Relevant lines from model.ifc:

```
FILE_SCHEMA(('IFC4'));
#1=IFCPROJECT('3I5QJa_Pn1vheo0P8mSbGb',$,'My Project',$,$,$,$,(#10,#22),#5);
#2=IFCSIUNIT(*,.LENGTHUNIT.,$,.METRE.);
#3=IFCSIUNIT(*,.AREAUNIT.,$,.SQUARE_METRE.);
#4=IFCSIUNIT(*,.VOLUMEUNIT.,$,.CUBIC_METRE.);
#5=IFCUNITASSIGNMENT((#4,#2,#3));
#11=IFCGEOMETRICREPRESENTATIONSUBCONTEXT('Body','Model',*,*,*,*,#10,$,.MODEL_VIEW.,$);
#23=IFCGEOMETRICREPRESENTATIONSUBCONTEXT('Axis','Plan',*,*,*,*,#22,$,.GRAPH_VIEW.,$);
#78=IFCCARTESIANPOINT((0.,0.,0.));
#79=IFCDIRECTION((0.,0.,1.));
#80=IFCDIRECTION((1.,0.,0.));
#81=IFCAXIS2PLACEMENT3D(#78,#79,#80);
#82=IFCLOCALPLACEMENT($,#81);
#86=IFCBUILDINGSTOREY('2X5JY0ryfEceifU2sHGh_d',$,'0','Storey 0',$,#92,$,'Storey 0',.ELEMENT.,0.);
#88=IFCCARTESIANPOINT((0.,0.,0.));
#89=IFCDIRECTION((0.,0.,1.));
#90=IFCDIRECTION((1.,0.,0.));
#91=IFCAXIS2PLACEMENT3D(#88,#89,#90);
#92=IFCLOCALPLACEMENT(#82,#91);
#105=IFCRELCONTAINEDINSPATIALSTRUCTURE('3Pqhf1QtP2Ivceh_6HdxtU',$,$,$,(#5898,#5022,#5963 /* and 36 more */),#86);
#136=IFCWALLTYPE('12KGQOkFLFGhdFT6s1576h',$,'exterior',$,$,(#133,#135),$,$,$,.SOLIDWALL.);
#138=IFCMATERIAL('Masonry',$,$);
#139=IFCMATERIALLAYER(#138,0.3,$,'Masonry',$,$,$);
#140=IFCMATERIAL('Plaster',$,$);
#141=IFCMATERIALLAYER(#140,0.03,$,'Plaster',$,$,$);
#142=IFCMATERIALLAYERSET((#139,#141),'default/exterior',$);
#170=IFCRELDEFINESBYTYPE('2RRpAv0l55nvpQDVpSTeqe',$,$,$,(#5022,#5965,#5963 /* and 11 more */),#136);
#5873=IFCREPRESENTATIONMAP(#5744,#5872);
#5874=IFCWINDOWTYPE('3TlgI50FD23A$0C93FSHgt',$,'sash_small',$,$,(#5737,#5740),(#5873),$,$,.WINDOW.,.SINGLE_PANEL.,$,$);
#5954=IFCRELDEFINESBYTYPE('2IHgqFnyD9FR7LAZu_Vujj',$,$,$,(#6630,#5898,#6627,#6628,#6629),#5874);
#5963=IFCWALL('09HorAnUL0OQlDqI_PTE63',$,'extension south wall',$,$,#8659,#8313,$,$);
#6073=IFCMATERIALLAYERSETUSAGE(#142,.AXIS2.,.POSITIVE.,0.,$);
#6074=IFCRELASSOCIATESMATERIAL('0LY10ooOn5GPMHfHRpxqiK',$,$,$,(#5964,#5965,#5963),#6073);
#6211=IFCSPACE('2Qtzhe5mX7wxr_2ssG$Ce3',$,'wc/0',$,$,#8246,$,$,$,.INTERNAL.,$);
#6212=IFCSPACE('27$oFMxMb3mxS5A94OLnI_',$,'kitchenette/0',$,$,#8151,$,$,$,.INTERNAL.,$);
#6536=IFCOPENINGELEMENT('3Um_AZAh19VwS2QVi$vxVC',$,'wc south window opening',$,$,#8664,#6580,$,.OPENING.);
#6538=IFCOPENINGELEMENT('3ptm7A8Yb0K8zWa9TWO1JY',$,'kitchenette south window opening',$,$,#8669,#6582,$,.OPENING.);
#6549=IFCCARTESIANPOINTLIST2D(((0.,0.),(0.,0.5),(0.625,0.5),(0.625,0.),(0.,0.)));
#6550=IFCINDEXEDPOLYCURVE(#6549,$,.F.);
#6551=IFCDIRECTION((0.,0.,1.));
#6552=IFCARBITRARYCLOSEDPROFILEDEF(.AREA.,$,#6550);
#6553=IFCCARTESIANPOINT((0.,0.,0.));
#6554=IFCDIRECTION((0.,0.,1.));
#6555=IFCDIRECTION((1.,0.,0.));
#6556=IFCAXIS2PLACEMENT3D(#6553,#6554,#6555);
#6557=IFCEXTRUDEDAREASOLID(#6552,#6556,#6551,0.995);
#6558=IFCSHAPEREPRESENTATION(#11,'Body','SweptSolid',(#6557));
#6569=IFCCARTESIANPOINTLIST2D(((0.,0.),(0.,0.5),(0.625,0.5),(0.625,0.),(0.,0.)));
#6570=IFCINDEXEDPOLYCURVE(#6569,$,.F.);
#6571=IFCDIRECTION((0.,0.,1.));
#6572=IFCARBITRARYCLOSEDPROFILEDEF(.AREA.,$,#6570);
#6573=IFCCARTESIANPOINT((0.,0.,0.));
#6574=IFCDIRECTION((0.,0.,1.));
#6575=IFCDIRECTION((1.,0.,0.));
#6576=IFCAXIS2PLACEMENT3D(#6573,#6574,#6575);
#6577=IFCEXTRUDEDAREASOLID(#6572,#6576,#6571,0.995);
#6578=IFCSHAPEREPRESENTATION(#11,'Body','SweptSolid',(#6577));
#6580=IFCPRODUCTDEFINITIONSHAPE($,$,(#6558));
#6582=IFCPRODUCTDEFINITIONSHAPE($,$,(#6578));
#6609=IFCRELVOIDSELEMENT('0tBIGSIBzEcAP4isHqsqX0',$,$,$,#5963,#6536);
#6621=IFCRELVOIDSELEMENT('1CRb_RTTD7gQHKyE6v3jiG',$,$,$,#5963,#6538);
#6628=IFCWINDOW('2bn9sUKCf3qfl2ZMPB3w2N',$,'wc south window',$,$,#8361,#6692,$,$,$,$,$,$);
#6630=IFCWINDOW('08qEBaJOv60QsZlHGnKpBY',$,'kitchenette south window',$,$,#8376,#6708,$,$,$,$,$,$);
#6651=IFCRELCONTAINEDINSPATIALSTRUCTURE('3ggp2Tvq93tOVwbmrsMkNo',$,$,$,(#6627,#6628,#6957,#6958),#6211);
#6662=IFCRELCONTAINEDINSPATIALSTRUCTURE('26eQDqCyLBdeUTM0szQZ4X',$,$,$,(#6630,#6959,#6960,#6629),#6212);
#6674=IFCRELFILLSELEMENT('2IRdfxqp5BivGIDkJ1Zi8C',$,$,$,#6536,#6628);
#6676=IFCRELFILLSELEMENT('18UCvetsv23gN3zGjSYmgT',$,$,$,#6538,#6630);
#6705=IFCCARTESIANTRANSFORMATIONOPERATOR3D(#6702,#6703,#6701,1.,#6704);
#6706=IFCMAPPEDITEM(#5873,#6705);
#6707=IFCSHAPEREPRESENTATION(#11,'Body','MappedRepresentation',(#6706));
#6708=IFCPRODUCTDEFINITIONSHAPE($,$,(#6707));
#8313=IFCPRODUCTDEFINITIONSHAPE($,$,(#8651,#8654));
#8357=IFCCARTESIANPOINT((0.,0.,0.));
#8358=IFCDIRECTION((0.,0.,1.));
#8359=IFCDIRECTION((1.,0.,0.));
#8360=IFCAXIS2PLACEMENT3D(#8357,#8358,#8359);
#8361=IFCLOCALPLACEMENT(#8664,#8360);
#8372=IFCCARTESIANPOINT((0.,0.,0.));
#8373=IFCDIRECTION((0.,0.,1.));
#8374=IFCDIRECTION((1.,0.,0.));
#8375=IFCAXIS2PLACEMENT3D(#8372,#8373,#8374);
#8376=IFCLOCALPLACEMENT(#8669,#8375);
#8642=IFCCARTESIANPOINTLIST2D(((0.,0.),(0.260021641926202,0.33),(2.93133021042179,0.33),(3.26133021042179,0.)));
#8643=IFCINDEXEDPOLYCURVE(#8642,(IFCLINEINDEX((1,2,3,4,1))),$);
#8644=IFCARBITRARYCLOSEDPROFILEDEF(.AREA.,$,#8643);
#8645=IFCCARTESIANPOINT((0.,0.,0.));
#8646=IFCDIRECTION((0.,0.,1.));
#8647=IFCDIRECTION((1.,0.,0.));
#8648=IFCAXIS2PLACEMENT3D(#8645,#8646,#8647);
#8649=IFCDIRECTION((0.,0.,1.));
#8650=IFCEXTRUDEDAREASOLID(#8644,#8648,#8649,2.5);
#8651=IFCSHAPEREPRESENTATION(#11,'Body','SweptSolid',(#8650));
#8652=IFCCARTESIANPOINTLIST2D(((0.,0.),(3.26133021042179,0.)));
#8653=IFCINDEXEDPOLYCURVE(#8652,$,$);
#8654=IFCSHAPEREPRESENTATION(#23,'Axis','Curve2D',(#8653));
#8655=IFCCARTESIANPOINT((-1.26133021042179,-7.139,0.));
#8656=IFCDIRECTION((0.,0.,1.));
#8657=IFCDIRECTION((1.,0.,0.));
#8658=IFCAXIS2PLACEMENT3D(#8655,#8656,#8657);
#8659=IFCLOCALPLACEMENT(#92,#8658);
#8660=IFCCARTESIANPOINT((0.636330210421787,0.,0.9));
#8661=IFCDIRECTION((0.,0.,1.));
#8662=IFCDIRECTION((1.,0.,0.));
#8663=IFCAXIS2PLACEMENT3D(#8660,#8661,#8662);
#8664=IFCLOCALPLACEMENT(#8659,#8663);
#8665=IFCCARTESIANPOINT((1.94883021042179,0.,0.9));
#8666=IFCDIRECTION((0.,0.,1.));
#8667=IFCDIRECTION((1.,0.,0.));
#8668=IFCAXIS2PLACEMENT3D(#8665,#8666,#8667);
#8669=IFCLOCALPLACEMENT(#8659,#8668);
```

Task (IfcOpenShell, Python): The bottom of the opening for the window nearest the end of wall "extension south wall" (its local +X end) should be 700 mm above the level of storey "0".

```python
import numpy as np
import ifcopenshell
import ifcopenshell.api.geometry
import ifcopenshell.geom
import ifcopenshell.util.element
import ifcopenshell.util.placement
import ifcopenshell.util.shape
import ifcopenshell.util.unit

model = ifcopenshell.open("model.ifc")
unit_scale = ifcopenshell.util.unit.calculate_unit_scale(model)

window = model.by_guid("08qEBaJOv60QsZlHGnKpBY")
opening = window.FillsVoids[0].RelatingOpeningElement
storey = ifcopenshell.util.element.get_container(window, ifc_class="IfcBuildingStorey")
level = ifcopenshell.util.placement.get_local_placement(storey.ObjectPlacement)[2, 3]

# The opening's origin need not be at the sill, so measure its lowest point.
shape = ifcopenshell.geom.create_shape(ifcopenshell.geom.settings(), opening)
bottom = ifcopenshell.util.shape.get_shape_bottom_elevation(shape, shape.geometry) / unit_scale
dz = level + 0.7 / unit_scale - bottom

shift = np.array([0.0, 0.0, dz])
# The window is placed relative to its opening, so it follows when the opening moves.
matrix = ifcopenshell.util.placement.get_local_placement(opening.ObjectPlacement)
matrix[:3, 3] += shift
ifcopenshell.api.geometry.edit_object_placement(
    model, product=opening, matrix=matrix, is_si=False, should_transform_children=True
)

print(f"moved by {dz * unit_scale:+.3f} m")

model.write("model_edited.ifc")
```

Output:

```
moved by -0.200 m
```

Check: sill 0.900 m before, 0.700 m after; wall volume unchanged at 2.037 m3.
